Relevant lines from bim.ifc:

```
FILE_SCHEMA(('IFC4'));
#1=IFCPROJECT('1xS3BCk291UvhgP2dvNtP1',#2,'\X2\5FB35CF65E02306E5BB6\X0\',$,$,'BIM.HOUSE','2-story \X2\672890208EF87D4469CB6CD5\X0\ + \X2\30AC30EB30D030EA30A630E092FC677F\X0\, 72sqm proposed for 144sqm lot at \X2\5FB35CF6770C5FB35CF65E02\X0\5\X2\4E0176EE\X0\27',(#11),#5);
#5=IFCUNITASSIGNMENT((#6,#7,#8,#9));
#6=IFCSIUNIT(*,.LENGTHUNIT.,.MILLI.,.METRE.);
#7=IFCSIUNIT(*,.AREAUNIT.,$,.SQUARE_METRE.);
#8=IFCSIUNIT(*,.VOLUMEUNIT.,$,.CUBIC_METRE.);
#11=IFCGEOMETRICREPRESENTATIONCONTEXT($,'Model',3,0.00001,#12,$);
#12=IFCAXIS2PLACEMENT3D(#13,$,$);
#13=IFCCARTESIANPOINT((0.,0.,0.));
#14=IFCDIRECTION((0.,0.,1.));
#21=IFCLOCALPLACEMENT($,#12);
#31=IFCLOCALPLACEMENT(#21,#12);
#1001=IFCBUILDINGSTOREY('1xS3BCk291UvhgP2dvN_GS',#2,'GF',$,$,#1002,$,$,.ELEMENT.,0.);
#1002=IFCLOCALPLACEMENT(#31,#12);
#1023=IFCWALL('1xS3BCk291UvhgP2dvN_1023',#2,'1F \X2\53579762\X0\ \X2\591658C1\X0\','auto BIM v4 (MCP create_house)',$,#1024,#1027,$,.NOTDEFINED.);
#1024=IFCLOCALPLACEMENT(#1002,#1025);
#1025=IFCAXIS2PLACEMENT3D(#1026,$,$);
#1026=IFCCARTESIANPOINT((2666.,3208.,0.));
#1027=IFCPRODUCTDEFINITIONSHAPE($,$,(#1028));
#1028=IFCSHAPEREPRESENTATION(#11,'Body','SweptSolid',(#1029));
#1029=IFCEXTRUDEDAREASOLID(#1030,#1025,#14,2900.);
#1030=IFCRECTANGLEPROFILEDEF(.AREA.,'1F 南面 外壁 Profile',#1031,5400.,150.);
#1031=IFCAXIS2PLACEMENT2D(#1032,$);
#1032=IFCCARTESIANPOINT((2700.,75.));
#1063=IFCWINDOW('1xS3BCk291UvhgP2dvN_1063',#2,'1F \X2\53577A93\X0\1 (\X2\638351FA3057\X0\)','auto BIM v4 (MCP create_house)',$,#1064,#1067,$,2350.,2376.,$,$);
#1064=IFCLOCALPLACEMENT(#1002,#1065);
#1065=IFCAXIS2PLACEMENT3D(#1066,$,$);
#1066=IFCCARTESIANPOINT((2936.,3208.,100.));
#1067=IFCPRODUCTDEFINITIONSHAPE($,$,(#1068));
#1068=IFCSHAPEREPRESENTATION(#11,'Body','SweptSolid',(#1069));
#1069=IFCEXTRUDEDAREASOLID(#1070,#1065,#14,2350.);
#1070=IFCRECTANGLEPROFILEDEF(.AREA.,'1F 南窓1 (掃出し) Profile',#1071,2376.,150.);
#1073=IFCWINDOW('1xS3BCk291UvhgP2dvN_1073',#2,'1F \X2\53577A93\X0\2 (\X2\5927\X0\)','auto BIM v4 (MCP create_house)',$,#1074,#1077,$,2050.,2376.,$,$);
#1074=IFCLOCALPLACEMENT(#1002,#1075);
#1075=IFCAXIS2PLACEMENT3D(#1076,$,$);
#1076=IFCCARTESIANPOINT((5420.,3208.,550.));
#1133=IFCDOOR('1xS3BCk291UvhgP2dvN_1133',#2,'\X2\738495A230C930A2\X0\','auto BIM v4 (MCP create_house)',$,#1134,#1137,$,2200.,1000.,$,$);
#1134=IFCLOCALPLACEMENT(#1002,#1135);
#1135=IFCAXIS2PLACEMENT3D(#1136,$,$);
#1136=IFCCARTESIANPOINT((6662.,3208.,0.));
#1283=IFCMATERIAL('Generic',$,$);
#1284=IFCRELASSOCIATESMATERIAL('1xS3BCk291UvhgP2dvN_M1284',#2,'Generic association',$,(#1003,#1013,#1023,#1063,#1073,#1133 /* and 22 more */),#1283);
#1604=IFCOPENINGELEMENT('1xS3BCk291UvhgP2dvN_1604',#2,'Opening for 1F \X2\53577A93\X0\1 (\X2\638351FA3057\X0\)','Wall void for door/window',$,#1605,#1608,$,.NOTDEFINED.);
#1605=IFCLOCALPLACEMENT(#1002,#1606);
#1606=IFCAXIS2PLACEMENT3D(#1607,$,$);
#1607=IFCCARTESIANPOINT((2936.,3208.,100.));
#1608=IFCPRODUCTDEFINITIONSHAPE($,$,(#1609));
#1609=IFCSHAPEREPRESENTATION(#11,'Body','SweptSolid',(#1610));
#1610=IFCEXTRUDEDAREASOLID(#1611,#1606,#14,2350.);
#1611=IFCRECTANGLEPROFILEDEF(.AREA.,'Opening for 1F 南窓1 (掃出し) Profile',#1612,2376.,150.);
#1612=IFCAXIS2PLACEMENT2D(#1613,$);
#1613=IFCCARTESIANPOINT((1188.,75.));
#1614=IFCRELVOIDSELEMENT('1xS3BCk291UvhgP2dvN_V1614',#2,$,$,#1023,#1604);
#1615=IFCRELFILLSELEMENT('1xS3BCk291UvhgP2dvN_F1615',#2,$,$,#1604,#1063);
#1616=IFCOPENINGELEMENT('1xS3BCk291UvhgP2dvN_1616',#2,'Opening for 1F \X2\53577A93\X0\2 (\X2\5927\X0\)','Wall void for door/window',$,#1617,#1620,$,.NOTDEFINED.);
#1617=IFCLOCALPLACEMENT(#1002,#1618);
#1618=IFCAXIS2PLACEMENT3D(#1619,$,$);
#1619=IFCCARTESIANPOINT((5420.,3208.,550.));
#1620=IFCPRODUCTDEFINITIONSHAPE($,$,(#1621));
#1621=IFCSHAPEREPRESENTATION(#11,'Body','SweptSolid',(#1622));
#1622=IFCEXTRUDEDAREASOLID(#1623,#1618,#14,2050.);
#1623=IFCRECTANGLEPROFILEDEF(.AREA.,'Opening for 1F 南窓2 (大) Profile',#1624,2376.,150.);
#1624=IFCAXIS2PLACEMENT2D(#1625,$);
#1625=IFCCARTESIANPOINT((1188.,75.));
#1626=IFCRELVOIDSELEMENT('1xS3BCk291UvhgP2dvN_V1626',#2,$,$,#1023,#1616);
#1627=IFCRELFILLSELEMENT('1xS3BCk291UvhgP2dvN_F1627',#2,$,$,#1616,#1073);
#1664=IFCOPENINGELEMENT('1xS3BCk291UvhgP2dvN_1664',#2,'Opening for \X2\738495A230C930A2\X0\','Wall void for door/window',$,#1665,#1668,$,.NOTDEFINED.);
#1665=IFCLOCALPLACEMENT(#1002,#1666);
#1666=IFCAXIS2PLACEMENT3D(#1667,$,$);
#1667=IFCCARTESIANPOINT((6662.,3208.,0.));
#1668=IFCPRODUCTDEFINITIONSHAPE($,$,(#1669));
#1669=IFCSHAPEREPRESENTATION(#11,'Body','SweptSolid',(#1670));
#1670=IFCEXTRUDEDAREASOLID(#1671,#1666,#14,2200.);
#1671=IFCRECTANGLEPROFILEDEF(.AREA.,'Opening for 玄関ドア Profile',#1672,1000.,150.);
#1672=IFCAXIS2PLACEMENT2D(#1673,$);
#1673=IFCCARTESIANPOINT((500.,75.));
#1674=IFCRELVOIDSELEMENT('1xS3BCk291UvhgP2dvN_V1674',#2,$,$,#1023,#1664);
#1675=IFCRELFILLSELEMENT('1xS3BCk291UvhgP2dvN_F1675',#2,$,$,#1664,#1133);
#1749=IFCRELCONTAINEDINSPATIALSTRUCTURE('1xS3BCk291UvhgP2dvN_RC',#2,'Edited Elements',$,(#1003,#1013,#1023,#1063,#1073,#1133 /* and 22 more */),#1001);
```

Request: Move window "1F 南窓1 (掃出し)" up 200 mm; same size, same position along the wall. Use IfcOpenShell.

```python
import numpy as np
import ifcopenshell
import ifcopenshell.api.geometry
import ifcopenshell.util.placement
import ifcopenshell.util.unit

model = ifcopenshell.open("bim.ifc")
unit_scale = ifcopenshell.util.unit.calculate_unit_scale(model)

window = model.by_id(1063)
opening = window.FillsVoids[0].RelatingOpeningElement
dz = 200.0

shift = np.array([0.0, 0.0, dz])
# The window is not placed relative to its opening, so move both.
for product in (opening, window):
    matrix = ifcopenshell.util.placement.get_local_placement(product.ObjectPlacement)
    matrix[:3, 3] += shift
    ifcopenshell.api.geometry.edit_object_placement(model, product=product, matrix=matrix, is_si=False)

print(f"moved by {dz * unit_scale:+.3f} m")

model.write("bim_rev.ifc")
```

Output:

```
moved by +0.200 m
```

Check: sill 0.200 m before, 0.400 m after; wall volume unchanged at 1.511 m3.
